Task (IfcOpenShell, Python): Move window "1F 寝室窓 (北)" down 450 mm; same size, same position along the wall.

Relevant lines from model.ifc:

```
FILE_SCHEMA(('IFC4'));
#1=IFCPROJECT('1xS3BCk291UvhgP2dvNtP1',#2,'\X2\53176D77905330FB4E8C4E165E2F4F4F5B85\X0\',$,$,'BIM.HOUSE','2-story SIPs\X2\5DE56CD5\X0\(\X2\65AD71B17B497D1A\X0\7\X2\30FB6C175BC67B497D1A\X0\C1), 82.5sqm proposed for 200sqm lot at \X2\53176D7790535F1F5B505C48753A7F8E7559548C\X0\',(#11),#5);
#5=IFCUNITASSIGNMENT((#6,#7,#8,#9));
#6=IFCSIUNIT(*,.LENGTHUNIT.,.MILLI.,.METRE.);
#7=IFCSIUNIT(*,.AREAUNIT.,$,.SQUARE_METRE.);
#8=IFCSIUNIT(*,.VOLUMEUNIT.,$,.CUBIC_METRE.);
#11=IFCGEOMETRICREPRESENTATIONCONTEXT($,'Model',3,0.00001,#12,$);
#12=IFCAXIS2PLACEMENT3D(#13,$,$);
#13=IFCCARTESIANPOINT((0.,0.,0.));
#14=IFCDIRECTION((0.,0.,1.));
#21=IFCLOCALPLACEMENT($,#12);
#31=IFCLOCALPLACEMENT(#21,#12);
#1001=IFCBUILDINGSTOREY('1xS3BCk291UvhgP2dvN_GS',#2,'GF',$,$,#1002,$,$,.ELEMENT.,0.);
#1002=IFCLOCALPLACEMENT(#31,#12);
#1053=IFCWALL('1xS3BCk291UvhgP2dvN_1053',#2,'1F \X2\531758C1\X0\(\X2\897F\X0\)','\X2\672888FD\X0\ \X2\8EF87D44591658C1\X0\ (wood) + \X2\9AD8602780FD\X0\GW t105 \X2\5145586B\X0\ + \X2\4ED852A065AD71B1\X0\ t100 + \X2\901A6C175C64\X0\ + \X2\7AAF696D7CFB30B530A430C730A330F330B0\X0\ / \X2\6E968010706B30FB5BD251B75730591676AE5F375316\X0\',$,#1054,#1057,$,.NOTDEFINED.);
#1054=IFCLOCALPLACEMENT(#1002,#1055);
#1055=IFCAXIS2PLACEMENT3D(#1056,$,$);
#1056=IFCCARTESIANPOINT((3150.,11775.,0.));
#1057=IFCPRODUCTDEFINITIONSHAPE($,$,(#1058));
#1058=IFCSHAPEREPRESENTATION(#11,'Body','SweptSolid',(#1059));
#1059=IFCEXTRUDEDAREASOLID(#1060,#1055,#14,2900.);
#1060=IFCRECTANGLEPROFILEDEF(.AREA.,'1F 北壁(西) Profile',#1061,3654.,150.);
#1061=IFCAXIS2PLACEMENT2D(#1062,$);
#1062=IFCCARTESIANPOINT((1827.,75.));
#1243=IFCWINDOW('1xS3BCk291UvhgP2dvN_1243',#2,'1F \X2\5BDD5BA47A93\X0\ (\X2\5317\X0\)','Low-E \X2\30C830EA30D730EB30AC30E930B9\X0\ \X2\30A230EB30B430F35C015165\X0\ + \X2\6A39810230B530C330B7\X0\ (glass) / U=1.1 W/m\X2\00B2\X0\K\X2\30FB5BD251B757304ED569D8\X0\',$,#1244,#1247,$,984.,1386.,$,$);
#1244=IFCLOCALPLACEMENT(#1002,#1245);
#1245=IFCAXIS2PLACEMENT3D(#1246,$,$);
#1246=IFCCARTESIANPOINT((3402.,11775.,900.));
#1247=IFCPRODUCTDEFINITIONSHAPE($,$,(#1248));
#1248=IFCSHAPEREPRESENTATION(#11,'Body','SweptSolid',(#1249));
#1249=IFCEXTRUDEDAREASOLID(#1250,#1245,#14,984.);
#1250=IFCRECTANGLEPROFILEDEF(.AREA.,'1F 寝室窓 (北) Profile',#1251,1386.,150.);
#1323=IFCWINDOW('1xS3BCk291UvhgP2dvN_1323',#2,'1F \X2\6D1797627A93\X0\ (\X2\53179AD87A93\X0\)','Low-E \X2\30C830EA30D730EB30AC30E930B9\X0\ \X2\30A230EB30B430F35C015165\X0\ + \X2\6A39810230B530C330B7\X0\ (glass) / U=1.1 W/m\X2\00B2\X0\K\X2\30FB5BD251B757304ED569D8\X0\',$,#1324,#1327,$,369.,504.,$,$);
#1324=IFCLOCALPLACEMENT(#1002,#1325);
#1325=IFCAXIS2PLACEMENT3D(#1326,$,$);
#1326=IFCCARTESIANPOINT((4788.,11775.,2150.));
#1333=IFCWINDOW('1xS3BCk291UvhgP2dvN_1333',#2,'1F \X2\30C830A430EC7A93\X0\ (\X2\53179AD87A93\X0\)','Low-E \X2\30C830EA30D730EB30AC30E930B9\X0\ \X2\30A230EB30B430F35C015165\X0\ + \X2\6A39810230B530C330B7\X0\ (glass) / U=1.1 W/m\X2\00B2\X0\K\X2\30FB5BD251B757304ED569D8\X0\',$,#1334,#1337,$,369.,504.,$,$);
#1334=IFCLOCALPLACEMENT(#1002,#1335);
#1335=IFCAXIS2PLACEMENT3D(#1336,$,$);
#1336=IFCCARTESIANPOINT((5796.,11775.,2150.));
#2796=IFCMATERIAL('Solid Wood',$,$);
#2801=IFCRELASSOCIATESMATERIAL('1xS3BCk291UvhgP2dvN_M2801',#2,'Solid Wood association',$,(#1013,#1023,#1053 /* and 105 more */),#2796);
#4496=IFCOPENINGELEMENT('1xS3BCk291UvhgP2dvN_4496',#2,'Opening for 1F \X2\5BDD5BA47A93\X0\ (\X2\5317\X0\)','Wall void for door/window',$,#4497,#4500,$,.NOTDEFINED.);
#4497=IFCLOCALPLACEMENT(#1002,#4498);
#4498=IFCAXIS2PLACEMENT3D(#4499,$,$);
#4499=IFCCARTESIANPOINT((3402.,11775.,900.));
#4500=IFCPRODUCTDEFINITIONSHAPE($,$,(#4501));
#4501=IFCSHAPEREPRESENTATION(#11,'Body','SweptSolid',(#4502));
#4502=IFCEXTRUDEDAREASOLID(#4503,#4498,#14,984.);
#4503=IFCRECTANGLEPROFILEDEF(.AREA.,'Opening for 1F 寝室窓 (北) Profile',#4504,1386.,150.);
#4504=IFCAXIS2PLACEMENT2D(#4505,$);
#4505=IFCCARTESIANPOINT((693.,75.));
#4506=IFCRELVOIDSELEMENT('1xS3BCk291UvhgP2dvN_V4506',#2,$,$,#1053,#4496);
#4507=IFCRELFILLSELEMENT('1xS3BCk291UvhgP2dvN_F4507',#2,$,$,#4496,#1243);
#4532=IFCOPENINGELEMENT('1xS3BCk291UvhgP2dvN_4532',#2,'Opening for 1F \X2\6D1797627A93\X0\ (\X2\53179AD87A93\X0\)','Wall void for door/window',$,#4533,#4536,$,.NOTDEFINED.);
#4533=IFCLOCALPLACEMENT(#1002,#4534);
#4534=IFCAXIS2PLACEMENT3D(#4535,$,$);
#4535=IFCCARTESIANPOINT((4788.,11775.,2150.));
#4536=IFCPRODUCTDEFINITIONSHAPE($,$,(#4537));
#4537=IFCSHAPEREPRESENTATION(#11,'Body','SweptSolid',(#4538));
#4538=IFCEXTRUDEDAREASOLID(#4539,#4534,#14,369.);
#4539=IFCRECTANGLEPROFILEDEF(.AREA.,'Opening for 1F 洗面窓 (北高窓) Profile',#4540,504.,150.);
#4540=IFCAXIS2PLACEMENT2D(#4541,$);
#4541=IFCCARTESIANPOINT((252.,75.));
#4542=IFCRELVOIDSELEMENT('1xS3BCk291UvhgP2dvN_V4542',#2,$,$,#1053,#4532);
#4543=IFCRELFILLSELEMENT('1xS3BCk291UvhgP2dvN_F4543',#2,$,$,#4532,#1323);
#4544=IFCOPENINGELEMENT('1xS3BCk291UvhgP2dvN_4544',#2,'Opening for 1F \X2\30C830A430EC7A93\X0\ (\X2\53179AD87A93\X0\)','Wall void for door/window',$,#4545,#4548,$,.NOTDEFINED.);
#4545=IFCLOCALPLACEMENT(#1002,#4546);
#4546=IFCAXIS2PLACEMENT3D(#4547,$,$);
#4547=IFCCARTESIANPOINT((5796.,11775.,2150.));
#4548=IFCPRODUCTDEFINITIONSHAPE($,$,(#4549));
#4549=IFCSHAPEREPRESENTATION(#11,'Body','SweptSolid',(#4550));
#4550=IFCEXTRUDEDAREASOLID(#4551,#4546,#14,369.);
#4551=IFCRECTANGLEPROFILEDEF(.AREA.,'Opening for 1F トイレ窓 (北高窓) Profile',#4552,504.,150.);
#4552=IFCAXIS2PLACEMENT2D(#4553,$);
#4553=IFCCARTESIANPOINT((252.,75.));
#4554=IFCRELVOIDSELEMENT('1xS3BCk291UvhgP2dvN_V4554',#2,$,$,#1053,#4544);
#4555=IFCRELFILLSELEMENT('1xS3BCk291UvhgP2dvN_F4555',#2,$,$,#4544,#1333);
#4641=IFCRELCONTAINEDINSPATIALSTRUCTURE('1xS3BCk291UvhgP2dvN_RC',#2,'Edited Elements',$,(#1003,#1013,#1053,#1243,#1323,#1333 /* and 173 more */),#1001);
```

```python
import numpy as np
import ifcopenshell
import ifcopenshell.api.geometry
import ifcopenshell.util.placement
import ifcopenshell.util.unit

model = ifcopenshell.open("model.ifc")
unit_scale = ifcopenshell.util.unit.calculate_unit_scale(model)

window = model.by_guid("1xS3BCk291UvhgP2dvN_1243")
opening = window.FillsVoids[0].RelatingOpeningElement
dz = -450.0

shift = np.array([0.0, 0.0, dz])
# The window is not placed relative to its opening, so move both.
for product in (opening, window):
    matrix = ifcopenshell.util.placement.get_local_placement(product.ObjectPlacement)
    matrix[:3, 3] += shift
    ifcopenshell.api.geometry.edit_object_placement(model, product=product, matrix=matrix, is_si=False)

print(f"moved by {dz * unit_scale:+.3f} m")

model.write("model_edited.ifc")
```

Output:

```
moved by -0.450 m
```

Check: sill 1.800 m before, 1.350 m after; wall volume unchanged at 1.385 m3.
